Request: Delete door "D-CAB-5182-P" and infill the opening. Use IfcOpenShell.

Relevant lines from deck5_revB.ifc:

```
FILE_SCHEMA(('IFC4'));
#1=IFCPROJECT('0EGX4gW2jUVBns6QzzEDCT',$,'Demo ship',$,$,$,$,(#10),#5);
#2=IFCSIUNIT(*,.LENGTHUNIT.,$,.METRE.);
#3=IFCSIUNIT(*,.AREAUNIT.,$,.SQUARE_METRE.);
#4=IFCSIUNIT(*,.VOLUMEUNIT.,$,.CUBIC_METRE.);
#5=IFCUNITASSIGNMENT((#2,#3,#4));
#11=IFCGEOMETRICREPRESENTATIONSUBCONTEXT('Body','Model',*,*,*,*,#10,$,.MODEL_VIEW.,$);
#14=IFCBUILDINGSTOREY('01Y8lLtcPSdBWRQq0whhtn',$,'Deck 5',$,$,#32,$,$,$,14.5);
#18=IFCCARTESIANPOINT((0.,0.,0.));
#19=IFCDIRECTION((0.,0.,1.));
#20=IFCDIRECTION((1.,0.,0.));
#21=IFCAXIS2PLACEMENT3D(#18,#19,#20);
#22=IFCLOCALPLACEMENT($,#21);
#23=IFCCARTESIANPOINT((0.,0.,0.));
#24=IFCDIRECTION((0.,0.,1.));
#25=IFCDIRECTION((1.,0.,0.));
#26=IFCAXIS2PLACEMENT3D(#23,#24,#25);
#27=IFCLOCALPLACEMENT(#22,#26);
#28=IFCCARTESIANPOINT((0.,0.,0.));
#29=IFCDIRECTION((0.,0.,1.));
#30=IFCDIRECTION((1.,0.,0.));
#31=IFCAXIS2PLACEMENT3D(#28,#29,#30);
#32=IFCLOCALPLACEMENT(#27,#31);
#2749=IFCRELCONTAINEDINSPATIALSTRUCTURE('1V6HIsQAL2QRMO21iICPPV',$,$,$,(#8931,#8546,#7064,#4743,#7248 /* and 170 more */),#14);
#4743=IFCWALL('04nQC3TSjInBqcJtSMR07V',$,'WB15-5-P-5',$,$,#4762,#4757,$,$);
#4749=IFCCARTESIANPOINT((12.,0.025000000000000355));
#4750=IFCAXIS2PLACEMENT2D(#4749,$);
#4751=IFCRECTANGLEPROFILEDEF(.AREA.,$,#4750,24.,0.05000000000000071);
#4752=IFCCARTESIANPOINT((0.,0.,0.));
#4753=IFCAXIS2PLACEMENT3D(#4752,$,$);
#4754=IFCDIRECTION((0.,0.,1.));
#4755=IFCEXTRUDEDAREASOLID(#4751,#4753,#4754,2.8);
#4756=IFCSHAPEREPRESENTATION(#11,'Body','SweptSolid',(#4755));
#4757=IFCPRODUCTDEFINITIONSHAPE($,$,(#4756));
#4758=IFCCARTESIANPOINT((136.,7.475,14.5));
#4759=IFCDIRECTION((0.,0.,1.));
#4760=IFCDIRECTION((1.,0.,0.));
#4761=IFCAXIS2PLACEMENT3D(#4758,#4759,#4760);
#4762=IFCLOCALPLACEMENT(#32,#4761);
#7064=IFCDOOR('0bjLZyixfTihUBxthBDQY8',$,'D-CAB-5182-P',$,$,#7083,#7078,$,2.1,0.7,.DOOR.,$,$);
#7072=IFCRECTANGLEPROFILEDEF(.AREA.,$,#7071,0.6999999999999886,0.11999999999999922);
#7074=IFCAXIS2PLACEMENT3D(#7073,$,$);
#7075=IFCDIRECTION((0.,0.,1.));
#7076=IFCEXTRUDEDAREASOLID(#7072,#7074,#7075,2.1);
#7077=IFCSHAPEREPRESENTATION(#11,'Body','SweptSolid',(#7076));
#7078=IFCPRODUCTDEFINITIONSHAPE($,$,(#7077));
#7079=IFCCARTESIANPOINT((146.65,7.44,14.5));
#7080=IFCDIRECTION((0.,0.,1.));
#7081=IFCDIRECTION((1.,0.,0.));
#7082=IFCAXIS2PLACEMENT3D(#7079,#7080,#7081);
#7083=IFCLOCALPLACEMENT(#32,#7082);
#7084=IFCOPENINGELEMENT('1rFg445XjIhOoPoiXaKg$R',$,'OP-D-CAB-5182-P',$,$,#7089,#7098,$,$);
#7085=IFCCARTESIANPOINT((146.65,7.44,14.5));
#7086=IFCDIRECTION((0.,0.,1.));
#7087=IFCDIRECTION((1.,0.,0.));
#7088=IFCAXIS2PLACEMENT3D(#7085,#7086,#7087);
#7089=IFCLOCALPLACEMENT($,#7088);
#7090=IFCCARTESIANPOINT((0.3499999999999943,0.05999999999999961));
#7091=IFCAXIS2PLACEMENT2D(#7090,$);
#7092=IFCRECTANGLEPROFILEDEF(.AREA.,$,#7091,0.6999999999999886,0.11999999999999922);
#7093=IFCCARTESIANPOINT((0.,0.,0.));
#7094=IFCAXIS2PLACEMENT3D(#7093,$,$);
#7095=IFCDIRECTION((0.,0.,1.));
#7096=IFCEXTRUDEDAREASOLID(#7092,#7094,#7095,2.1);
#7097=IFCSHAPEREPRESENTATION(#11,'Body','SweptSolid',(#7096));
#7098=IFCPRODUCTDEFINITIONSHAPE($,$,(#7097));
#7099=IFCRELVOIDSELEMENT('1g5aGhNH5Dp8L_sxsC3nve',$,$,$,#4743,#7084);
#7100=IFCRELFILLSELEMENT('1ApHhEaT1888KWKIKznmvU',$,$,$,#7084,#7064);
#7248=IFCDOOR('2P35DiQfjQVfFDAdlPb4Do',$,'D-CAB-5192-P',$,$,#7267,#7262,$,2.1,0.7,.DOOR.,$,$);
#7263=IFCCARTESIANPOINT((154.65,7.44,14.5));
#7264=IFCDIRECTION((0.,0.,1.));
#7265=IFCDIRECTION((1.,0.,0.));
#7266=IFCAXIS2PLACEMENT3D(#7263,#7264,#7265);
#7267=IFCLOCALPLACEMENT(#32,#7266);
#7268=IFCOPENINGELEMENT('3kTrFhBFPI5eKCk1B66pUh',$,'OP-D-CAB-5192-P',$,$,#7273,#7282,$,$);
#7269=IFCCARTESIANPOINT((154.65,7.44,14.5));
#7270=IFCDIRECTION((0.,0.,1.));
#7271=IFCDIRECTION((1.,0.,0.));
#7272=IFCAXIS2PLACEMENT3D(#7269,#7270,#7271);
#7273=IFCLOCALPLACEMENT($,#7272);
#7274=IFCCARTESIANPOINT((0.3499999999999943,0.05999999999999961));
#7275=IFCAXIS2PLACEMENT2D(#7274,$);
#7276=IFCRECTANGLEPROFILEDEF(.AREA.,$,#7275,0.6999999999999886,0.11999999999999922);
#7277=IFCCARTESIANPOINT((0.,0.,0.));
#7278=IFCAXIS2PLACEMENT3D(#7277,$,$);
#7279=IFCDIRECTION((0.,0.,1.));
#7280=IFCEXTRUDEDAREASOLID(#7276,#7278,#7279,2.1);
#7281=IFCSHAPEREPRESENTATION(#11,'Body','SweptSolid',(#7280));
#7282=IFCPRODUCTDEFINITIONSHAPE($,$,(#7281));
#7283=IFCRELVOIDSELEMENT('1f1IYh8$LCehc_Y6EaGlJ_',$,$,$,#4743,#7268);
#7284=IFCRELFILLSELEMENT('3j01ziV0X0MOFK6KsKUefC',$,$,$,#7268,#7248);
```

```python
import ifcopenshell
import ifcopenshell.api.feature
import ifcopenshell.api.root
import ifcopenshell.geom
import ifcopenshell.util.shape

model = ifcopenshell.open("deck5_revB.ifc")
settings = ifcopenshell.geom.settings()


def volume(element):
    """Net volume in cubic metres, openings subtracted."""
    shape = ifcopenshell.geom.create_shape(settings, element)
    return ifcopenshell.util.shape.get_volume(shape.geometry)


door = model.by_id(7064)
opening = door.FillsVoids[0].RelatingOpeningElement
wall = opening.VoidsElements[0].RelatingBuildingElement
before = volume(wall)

ifcopenshell.api.root.remove_product(model, product=door)
ifcopenshell.api.feature.remove_feature(model, feature=opening)

after = volume(wall)

print(f"wall volume {before:.3f} -> {after:.3f} m3")

model.write("deck5_revB-out.ifc")
```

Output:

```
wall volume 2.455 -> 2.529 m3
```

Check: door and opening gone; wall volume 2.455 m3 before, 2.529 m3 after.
